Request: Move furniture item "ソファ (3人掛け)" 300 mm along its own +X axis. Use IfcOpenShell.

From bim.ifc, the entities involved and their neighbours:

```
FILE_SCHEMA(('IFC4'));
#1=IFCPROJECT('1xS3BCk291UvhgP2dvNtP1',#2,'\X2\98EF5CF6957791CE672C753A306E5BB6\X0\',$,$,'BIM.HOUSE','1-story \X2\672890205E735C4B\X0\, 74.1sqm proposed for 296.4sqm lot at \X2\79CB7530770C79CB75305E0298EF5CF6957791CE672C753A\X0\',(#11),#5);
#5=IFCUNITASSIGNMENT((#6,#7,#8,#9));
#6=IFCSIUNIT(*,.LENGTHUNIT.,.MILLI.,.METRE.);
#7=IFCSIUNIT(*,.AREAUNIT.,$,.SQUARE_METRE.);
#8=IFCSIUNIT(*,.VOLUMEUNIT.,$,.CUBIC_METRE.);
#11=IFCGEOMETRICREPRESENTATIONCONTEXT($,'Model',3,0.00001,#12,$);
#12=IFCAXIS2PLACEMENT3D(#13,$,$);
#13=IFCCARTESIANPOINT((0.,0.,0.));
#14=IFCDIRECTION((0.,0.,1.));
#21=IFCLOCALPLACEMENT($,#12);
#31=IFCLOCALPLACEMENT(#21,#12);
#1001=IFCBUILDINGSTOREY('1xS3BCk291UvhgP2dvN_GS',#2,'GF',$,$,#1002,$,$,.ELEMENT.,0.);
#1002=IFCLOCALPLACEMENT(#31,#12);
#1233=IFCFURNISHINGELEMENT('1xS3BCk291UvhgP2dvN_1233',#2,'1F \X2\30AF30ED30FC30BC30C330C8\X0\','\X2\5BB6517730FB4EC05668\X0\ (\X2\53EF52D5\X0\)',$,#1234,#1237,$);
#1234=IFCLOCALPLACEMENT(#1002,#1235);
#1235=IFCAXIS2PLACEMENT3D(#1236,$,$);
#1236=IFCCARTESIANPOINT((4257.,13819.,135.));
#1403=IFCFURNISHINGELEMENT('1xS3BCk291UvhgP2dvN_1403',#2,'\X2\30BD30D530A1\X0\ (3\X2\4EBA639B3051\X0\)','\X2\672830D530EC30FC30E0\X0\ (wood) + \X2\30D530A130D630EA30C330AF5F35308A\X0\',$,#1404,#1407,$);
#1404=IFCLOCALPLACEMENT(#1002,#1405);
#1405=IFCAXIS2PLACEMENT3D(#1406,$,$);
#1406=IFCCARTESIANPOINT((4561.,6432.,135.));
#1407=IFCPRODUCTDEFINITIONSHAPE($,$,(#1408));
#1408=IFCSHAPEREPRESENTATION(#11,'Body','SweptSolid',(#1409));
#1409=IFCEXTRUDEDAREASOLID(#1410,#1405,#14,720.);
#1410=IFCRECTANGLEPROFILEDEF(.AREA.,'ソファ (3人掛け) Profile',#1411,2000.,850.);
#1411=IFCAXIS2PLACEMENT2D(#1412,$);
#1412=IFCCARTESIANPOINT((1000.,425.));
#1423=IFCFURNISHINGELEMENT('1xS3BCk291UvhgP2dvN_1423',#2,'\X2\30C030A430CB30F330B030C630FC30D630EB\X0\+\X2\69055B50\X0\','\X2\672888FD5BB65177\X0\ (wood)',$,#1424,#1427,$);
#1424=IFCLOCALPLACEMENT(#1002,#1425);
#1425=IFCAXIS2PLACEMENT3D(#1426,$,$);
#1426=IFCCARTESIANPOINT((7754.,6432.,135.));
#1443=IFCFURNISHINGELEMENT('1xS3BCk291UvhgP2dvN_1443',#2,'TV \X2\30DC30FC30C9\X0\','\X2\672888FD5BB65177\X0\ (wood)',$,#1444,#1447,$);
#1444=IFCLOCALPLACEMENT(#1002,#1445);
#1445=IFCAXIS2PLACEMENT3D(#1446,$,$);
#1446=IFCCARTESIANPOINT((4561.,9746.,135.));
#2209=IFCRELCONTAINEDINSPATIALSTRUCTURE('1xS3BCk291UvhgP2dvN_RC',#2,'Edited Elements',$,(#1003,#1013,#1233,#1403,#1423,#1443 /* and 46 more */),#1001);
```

```python
import ifcopenshell
import ifcopenshell.api.geometry
import ifcopenshell.util.placement
import ifcopenshell.util.unit

model = ifcopenshell.open("bim.ifc")
unit_scale = ifcopenshell.util.unit.calculate_unit_scale(model)

item = model.by_guid("1xS3BCk291UvhgP2dvN_1403")
matrix = ifcopenshell.util.placement.get_local_placement(item.ObjectPlacement)
matrix[:3, 3] += matrix[:3, 0] * 0.3 / unit_scale
ifcopenshell.api.geometry.edit_object_placement(model, product=item, matrix=matrix, is_si=False)

print(ifcopenshell.util.placement.get_local_placement(item.ObjectPlacement).round(3) + 0.0)

model.write("bim-out.ifc")
```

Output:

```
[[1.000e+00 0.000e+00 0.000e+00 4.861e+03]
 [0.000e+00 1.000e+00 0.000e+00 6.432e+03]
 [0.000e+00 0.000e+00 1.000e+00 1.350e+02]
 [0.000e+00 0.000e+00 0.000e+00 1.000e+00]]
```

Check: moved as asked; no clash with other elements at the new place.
